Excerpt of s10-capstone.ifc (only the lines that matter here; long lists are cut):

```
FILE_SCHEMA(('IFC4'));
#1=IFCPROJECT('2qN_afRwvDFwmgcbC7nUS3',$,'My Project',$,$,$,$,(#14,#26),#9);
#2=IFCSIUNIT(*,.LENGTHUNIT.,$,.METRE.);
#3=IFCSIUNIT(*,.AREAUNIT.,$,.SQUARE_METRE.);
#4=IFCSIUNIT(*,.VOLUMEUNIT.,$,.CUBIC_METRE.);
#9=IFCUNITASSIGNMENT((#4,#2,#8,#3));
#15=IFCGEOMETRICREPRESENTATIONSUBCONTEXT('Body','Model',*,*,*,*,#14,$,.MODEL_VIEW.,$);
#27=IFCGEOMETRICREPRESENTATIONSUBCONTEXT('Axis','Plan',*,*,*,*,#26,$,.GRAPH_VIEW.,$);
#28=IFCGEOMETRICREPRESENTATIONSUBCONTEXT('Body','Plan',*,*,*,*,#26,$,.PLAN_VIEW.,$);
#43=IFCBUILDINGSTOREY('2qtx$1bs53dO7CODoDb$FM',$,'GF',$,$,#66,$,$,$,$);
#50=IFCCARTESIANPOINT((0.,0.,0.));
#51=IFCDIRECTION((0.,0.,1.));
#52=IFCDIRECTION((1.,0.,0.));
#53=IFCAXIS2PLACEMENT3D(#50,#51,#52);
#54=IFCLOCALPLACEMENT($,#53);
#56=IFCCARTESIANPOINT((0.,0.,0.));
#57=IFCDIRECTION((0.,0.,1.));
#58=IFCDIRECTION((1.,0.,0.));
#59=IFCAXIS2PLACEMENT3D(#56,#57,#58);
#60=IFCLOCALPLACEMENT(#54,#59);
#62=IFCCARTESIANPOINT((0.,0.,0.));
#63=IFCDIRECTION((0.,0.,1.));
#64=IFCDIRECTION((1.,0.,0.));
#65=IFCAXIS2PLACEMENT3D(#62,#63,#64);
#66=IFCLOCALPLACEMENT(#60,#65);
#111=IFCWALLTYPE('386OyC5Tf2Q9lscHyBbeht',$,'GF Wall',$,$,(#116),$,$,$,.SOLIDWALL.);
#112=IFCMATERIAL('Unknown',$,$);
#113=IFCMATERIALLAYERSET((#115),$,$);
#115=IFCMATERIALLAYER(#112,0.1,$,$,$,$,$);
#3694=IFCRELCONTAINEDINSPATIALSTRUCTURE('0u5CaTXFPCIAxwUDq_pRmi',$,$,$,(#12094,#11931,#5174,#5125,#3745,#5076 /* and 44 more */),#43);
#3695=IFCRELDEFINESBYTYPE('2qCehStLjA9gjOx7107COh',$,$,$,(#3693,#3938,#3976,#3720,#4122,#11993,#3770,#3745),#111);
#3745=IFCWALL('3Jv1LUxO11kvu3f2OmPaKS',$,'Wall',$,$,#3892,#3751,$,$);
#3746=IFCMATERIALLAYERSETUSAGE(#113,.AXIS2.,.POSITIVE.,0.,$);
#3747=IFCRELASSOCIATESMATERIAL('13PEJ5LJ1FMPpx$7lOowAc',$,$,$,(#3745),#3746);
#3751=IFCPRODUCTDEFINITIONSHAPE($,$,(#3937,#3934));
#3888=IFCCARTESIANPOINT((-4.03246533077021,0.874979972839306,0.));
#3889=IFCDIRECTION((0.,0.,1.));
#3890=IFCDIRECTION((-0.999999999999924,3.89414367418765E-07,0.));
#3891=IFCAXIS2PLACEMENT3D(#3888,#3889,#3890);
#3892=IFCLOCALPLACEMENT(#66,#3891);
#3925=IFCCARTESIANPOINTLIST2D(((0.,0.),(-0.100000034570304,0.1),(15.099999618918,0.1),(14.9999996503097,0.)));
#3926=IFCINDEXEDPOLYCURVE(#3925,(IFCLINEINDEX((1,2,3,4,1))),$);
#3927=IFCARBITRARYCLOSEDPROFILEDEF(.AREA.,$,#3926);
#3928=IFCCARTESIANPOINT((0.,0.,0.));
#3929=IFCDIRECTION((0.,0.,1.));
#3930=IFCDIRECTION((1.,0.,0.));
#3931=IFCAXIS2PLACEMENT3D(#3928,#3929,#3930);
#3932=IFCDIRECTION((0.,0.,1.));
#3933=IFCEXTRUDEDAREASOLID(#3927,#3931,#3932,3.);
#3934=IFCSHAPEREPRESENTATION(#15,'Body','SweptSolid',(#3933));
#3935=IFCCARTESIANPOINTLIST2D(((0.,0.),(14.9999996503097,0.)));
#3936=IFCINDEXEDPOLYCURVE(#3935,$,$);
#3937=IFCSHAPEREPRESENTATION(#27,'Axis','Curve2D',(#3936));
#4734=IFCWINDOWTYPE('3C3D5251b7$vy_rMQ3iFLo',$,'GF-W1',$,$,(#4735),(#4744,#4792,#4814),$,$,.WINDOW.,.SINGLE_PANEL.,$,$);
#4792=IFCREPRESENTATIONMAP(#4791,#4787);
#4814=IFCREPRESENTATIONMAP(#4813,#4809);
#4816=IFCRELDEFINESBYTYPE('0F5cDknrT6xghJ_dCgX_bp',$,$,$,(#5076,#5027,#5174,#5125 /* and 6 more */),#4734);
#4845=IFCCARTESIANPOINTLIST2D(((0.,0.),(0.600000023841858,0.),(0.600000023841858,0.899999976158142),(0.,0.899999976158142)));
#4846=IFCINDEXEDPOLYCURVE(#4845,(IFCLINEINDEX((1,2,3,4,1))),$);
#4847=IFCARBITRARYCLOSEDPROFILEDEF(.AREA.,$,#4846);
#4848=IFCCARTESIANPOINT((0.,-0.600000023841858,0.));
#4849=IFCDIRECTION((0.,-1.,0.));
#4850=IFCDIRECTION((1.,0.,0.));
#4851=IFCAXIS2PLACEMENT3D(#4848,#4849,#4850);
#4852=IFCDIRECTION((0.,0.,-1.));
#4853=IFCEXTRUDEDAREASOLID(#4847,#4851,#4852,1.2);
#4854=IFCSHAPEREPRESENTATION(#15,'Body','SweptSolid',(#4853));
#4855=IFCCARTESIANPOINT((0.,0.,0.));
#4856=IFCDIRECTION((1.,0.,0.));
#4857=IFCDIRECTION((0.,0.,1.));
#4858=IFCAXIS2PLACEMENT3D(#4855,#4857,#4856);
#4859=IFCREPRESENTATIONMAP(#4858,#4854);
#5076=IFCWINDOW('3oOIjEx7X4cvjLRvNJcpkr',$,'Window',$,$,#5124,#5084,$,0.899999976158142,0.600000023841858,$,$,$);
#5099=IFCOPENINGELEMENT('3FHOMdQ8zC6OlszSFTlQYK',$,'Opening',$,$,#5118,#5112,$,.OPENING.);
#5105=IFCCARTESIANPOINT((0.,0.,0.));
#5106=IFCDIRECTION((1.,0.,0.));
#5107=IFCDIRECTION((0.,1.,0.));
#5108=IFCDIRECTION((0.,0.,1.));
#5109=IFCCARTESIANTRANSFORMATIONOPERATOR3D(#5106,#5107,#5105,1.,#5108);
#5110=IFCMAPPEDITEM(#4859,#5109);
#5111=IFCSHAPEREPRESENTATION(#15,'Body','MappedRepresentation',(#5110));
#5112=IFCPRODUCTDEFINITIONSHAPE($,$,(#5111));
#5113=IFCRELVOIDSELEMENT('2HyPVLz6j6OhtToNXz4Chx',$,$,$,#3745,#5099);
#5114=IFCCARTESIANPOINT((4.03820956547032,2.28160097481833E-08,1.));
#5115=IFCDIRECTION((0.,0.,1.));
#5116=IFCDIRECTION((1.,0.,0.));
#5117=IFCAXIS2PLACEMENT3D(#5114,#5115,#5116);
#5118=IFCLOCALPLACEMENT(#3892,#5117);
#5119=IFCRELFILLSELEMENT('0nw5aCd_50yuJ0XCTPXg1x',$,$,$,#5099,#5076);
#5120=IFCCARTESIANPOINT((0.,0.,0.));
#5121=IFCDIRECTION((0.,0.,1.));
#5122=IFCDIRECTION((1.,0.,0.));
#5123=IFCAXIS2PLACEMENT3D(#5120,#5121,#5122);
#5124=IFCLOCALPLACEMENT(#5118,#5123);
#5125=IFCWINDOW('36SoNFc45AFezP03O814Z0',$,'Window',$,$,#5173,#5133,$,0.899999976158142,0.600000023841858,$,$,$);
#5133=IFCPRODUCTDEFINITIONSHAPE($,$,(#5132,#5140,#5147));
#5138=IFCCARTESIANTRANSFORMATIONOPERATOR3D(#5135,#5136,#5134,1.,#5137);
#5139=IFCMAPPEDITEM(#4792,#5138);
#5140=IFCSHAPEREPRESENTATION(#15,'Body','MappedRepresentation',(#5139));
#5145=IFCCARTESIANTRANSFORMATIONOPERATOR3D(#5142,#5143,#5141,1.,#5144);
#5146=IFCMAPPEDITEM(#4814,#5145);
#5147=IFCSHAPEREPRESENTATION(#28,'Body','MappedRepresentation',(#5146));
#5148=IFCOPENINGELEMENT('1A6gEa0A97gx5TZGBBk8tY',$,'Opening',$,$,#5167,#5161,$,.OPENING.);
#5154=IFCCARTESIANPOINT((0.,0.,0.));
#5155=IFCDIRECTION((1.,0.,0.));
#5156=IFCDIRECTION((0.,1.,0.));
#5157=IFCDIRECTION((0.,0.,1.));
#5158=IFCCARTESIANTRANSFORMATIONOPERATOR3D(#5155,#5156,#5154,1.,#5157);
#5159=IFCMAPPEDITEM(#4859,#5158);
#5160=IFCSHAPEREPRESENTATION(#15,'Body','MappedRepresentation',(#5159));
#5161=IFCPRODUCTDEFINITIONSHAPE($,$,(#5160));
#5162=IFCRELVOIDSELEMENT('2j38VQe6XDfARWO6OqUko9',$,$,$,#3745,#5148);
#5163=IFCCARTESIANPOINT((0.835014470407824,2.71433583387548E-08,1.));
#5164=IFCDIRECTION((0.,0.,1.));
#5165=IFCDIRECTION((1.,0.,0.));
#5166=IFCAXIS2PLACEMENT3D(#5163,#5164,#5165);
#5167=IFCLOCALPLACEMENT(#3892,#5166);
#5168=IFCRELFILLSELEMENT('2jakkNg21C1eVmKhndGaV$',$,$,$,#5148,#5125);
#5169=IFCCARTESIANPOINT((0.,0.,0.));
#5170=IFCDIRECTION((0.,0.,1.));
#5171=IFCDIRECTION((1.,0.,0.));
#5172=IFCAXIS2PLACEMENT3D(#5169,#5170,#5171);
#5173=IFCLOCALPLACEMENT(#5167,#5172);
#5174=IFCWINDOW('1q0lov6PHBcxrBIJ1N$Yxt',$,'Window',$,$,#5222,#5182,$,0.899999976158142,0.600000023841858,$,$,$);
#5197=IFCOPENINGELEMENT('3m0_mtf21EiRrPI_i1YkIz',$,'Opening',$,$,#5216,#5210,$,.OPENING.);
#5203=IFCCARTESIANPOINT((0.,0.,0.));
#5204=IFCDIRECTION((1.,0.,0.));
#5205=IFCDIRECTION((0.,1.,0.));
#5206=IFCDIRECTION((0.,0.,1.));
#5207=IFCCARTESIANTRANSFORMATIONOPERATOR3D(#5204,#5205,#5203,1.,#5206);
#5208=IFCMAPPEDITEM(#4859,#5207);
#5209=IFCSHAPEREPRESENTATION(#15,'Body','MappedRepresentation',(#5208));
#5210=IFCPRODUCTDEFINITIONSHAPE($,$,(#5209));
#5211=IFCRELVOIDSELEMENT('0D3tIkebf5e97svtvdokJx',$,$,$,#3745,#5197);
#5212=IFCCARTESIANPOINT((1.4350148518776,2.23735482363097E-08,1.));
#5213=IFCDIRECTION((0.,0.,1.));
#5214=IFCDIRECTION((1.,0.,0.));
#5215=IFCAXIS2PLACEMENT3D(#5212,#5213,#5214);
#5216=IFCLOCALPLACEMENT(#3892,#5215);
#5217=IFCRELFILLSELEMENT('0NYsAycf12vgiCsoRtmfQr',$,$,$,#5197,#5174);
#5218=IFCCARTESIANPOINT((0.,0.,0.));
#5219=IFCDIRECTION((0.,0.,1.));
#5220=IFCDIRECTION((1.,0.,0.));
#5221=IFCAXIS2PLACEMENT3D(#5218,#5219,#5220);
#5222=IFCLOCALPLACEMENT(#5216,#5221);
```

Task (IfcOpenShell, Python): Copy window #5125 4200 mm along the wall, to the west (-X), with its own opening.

```python
import ifcopenshell
import ifcopenshell.api.feature
import ifcopenshell.api.geometry
import ifcopenshell.api.root
import ifcopenshell.geom
import ifcopenshell.util.element
import ifcopenshell.util.placement
import ifcopenshell.util.shape

model = ifcopenshell.open("s10-capstone.ifc")
settings = ifcopenshell.geom.settings()


def volume(element):
    """Net volume in cubic metres, openings subtracted."""
    shape = ifcopenshell.geom.create_shape(settings, element)
    return ifcopenshell.util.shape.get_volume(shape.geometry)


window = model.by_id(5125)
opening = window.FillsVoids[0].RelatingOpeningElement
wall = opening.VoidsElements[0].RelatingBuildingElement
before = volume(wall)
shift = ifcopenshell.util.placement.get_local_placement(wall.ObjectPlacement)[:3, 0] * 4.2

# copy_class copies the void relationship, type, container and properties, but no geometry.
new_opening = ifcopenshell.api.root.copy_class(model, product=opening)
new_opening.Representation = ifcopenshell.util.element.copy_deep(
    model, opening.Representation, exclude=["IfcGeometricRepresentationContext", "IfcRepresentationMap"]
)
new_window = ifcopenshell.api.root.copy_class(model, product=window)
new_window.Representation = ifcopenshell.util.element.copy_deep(
    model, window.Representation, exclude=["IfcGeometricRepresentationContext", "IfcRepresentationMap"]
)
ifcopenshell.api.feature.add_filling(model, opening=new_opening, element=new_window)

for old, new in ((opening, new_opening), (window, new_window)):
    matrix = ifcopenshell.util.placement.get_local_placement(old.ObjectPlacement)
    matrix[:3, 3] += shift
    ifcopenshell.api.geometry.edit_object_placement(model, product=new, matrix=matrix, is_si=False)

after = volume(wall)

print(f"wall volume {before:.3f} -> {after:.3f} m3")

model.write("s10-capstone_updated.ifc")
```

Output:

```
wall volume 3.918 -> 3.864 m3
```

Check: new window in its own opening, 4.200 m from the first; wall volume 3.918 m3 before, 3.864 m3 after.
